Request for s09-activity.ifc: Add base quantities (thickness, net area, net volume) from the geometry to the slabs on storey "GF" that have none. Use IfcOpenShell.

First a look at what the model holds.

```python
import ifcopenshell
import ifcopenshell.util.element
import ifcopenshell.util.unit

model = ifcopenshell.open("s09-activity.ifc")
print(model.schema)
for unit_type in ("LENGTHUNIT", "AREAUNIT", "VOLUMEUNIT"):
    print(unit_type, ifcopenshell.util.unit.calculate_unit_scale(model, unit_type))
storey = next(s for s in model.by_type("IfcBuildingStorey") if s.Name == "GF")
slabs = [e for e in ifcopenshell.util.element.get_decomposition(storey) if e.is_a("IfcSlab")]
for e in sorted(slabs, key=lambda e: e.id()):
    print(e.id(), e.is_a(), e.Name, list(ifcopenshell.util.element.get_psets(e, qtos_only=True)), sep=" | ")
```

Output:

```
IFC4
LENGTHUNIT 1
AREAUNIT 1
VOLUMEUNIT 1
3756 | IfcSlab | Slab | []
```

```python
import ifcopenshell
import ifcopenshell.api.pset
import ifcopenshell.geom
import ifcopenshell.util.element
import ifcopenshell.util.shape
import ifcopenshell.util.unit

model = ifcopenshell.open("s09-activity.ifc")
unit_scale = ifcopenshell.util.unit.calculate_unit_scale(model)
area_scale = ifcopenshell.util.unit.calculate_unit_scale(model, "AREAUNIT")
volume_scale = ifcopenshell.util.unit.calculate_unit_scale(model, "VOLUMEUNIT")
settings = ifcopenshell.geom.settings()

storey = next(s for s in model.by_type("IfcBuildingStorey") if s.Name == "GF")
slabs = [e for e in ifcopenshell.util.element.get_decomposition(storey) if e.is_a("IfcSlab")]

for e in sorted(slabs, key=lambda e: e.id()):
    if ifcopenshell.util.element.get_psets(e, qtos_only=True, should_inherit=False):
        continue
    # Geometry comes back in metres, in the element's own axes.
    shape = ifcopenshell.geom.create_shape(settings, e)
    values = {
        "Width": ifcopenshell.util.shape.get_z(shape.geometry) / unit_scale,
        "NetArea": ifcopenshell.util.shape.get_footprint_area(shape.geometry) / area_scale,
        "NetVolume": ifcopenshell.util.shape.get_volume(shape.geometry) / volume_scale,
    }
    qto = ifcopenshell.api.pset.add_qto(model, product=e, name="Qto_SlabBaseQuantities")
    ifcopenshell.api.pset.edit_qto(model, qto=qto, properties=values)
    print(e.id(), {k: round(v, 3) for k, v in values.items()})

model.write("s09-activity_rev.ifc")
```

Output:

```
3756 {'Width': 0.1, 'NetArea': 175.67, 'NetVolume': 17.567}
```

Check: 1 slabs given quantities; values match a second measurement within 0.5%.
